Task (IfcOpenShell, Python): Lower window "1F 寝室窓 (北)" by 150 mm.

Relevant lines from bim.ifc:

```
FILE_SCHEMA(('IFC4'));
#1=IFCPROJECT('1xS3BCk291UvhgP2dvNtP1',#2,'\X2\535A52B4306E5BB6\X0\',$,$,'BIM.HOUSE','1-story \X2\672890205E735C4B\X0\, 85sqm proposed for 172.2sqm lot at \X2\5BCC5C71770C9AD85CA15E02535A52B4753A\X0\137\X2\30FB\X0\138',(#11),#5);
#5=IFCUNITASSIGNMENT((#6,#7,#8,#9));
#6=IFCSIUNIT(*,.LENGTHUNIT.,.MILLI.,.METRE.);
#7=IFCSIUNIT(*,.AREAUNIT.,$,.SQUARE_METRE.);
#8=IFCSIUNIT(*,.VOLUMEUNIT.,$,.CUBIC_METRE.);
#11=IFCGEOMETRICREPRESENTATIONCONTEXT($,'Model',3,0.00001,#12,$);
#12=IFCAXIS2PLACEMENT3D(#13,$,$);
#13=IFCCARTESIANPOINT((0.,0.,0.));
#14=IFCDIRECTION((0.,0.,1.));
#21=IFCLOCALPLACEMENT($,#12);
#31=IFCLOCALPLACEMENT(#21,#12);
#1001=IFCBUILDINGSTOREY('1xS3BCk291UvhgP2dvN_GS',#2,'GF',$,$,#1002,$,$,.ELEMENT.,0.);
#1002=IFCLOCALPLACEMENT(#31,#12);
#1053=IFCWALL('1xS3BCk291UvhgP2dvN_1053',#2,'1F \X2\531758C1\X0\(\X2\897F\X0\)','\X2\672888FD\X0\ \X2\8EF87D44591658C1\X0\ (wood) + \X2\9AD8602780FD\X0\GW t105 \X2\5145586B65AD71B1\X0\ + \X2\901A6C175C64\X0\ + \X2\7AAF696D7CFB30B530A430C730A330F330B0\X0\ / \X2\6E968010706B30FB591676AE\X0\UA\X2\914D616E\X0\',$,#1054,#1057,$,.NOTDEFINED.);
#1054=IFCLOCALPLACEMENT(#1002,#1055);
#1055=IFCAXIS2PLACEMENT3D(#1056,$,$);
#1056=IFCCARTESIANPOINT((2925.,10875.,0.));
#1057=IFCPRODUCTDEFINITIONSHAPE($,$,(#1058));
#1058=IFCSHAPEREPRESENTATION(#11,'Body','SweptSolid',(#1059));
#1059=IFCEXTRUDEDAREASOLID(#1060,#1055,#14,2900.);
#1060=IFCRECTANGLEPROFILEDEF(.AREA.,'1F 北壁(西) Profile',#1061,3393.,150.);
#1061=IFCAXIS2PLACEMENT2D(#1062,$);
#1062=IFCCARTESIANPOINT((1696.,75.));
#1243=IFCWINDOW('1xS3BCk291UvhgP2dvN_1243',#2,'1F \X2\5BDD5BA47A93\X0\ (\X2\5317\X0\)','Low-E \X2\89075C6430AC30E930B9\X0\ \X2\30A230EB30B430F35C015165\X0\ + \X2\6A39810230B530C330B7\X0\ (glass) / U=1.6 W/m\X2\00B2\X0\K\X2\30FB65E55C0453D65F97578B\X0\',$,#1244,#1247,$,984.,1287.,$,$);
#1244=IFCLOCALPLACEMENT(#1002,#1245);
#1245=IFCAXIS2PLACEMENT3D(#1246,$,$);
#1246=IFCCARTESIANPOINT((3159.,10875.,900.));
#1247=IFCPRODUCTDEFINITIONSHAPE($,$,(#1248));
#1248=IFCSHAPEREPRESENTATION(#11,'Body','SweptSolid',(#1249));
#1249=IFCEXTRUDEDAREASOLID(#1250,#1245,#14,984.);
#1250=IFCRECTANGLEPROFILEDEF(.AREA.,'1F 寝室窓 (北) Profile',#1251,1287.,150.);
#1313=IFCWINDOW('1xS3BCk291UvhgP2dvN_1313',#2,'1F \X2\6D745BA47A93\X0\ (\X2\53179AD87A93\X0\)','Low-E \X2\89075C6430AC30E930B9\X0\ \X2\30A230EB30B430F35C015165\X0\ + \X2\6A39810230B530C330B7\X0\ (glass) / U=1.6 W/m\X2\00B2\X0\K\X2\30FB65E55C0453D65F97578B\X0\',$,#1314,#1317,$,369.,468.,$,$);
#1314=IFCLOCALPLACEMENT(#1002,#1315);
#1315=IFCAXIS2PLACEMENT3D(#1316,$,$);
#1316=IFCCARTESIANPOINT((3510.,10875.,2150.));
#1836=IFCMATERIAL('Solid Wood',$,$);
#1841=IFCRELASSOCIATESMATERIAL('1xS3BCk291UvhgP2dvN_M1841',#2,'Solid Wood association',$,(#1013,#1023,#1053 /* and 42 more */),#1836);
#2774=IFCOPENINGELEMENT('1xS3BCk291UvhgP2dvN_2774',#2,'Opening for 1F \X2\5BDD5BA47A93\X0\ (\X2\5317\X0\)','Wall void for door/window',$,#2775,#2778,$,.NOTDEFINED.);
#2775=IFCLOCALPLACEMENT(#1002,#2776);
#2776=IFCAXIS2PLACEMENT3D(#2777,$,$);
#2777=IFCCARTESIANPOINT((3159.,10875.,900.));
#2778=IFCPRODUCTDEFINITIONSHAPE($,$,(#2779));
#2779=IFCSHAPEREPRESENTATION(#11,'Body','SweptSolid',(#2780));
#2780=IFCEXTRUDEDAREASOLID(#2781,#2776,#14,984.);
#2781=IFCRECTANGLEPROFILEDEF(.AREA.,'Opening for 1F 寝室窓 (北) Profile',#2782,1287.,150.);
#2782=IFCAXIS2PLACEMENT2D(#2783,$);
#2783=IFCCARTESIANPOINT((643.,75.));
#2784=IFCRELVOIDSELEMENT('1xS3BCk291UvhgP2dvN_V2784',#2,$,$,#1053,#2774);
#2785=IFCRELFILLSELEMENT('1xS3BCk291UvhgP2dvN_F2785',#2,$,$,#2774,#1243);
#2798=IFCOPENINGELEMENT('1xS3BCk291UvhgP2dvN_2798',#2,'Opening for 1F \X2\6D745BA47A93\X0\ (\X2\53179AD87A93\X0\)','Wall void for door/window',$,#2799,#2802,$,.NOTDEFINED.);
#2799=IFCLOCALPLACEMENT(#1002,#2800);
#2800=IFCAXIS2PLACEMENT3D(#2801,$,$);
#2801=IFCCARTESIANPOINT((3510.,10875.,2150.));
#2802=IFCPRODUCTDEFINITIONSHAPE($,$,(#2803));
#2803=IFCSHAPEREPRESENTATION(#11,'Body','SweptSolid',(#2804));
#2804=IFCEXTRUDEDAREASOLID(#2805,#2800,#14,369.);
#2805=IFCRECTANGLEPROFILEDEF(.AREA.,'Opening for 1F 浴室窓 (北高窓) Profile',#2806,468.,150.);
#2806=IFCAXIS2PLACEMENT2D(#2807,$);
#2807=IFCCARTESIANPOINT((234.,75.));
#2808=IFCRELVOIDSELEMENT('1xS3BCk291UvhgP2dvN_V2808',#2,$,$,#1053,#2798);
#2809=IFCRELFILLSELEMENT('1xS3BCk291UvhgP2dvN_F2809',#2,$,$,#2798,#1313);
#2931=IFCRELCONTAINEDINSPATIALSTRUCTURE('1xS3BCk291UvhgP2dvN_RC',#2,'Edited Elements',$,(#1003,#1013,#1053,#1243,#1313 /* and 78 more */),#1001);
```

```python
import numpy as np
import ifcopenshell
import ifcopenshell.api.geometry
import ifcopenshell.util.placement
import ifcopenshell.util.unit

model = ifcopenshell.open("bim.ifc")
unit_scale = ifcopenshell.util.unit.calculate_unit_scale(model)

window = model.by_guid("1xS3BCk291UvhgP2dvN_1243")
opening = window.FillsVoids[0].RelatingOpeningElement
dz = -0.15 / unit_scale

shift = np.array([0.0, 0.0, dz])
# The window is not placed relative to its opening, so move both.
for product in (opening, window):
    matrix = ifcopenshell.util.placement.get_local_placement(product.ObjectPlacement)
    matrix[:3, 3] += shift
    ifcopenshell.api.geometry.edit_object_placement(model, product=product, matrix=matrix, is_si=False)

print(f"moved by {dz * unit_scale:+.3f} m")

model.write("bim_rev.ifc")
```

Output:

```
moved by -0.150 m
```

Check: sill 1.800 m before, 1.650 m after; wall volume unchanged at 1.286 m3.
